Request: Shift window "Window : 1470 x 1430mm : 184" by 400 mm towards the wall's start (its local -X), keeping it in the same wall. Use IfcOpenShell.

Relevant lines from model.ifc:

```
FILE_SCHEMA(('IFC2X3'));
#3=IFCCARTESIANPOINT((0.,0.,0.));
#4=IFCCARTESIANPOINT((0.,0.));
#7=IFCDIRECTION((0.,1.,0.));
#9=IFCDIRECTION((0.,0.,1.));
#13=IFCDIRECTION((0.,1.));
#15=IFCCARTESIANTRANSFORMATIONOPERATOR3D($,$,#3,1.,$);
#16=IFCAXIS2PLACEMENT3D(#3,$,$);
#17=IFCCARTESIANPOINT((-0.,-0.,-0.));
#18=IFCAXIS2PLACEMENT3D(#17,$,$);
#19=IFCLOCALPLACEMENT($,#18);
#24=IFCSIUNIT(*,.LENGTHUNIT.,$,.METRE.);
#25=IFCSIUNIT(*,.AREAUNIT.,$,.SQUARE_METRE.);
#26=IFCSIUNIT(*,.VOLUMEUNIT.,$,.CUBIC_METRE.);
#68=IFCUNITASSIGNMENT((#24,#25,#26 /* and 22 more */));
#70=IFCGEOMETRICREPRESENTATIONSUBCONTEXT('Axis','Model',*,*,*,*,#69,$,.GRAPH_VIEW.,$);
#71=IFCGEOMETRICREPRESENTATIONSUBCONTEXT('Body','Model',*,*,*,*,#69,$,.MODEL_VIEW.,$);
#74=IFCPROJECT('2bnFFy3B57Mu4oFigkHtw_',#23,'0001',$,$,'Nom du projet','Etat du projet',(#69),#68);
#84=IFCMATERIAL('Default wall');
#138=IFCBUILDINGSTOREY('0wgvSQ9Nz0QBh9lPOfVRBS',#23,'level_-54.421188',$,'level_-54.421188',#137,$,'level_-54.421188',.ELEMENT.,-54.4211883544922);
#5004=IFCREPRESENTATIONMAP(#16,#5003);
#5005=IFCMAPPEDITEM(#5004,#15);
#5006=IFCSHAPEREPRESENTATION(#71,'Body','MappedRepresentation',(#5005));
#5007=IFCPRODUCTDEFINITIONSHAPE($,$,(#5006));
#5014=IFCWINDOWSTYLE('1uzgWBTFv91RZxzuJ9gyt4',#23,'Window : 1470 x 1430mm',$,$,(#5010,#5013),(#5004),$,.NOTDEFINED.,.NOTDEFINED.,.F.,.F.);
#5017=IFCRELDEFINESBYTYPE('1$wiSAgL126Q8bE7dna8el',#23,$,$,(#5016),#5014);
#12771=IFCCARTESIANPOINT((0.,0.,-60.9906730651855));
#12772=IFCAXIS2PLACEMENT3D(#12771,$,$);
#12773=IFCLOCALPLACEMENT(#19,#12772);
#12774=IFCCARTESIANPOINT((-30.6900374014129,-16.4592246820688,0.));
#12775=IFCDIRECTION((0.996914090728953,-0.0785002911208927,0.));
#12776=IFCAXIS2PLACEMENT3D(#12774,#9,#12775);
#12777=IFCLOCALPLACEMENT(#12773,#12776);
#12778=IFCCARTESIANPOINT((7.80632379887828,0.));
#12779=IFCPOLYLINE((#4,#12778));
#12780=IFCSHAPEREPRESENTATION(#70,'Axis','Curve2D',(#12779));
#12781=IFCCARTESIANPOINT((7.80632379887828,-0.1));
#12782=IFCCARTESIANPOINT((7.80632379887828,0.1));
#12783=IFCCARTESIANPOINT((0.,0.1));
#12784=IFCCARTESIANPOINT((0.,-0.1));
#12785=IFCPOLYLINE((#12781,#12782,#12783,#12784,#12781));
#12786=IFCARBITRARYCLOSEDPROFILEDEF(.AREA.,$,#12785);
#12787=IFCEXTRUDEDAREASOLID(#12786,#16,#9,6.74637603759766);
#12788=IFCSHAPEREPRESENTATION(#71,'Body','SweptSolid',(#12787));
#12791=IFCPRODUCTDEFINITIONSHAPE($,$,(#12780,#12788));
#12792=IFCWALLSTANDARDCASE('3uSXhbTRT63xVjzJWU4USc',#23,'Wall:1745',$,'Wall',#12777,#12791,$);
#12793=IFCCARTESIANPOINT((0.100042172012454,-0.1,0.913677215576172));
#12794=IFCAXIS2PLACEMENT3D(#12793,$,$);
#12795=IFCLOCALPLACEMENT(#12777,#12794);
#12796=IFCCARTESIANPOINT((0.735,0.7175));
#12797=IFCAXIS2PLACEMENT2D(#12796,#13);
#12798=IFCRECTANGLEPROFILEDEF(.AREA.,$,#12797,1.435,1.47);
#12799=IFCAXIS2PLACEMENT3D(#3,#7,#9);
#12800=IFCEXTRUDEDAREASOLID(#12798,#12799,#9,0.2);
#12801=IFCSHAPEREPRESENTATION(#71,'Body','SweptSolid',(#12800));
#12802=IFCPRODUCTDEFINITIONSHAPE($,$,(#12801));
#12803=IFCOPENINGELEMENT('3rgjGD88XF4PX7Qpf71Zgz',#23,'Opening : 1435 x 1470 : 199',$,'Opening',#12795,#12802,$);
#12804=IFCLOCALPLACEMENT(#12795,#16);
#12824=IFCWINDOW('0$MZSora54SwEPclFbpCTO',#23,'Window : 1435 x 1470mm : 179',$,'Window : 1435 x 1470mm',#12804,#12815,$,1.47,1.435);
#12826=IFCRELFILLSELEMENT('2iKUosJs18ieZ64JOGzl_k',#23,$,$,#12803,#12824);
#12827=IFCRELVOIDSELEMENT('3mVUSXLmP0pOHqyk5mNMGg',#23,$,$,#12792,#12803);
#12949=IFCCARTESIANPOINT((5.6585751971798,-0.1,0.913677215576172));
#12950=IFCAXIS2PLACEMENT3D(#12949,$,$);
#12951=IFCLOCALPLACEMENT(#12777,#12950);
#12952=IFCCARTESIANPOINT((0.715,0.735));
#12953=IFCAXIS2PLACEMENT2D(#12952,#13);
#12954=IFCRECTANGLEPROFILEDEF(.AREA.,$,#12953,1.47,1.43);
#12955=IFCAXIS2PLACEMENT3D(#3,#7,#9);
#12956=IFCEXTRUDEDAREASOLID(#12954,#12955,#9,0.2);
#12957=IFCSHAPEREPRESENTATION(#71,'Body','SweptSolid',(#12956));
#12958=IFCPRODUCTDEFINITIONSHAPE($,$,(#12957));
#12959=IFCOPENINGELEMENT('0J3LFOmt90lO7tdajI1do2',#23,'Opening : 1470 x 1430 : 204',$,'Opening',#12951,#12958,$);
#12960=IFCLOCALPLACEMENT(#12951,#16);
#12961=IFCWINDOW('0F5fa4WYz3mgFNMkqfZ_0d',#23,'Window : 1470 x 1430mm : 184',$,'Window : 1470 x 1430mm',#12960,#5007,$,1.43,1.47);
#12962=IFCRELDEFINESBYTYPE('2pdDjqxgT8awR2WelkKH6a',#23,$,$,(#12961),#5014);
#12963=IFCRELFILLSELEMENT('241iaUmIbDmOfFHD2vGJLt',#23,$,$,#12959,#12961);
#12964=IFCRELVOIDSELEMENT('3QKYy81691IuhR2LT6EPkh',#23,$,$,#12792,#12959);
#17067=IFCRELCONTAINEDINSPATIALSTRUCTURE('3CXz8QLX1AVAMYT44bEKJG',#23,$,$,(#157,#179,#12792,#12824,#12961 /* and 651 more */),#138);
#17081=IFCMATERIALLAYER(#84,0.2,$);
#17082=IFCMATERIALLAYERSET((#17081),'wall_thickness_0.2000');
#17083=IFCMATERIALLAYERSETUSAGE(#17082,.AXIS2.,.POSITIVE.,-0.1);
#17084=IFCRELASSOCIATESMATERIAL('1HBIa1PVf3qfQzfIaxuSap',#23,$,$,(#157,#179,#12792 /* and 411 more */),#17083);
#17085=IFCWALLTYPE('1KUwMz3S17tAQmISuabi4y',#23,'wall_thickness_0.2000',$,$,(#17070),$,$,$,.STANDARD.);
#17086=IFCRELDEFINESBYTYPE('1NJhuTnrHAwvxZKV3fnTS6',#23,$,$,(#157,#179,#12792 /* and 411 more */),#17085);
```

```python
import ifcopenshell
import ifcopenshell.api.geometry
import ifcopenshell.util.placement

model = ifcopenshell.open("model.ifc")

window = model.by_guid("0F5fa4WYz3mgFNMkqfZ_0d")
opening = window.FillsVoids[0].RelatingOpeningElement
wall = opening.VoidsElements[0].RelatingBuildingElement

wall_matrix = ifcopenshell.util.placement.get_local_placement(wall.ObjectPlacement)
shift = wall_matrix[:3, 0] * -0.4
before = ifcopenshell.util.placement.get_local_placement(window.ObjectPlacement)[:3, 3].copy()

# The window is placed relative to its opening, so it follows when the opening moves.
matrix = ifcopenshell.util.placement.get_local_placement(opening.ObjectPlacement)
matrix[:3, 3] += shift
ifcopenshell.api.geometry.edit_object_placement(
    model, product=opening, matrix=matrix, is_si=False, should_transform_children=True
)

after = ifcopenshell.util.placement.get_local_placement(window.ObjectPlacement)[:3, 3]
print("window moved by", (after - before).round(3) + 0.0)

model.write("model_updated.ifc")
```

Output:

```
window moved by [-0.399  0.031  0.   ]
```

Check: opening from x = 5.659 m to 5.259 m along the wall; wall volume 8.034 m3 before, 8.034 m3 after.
